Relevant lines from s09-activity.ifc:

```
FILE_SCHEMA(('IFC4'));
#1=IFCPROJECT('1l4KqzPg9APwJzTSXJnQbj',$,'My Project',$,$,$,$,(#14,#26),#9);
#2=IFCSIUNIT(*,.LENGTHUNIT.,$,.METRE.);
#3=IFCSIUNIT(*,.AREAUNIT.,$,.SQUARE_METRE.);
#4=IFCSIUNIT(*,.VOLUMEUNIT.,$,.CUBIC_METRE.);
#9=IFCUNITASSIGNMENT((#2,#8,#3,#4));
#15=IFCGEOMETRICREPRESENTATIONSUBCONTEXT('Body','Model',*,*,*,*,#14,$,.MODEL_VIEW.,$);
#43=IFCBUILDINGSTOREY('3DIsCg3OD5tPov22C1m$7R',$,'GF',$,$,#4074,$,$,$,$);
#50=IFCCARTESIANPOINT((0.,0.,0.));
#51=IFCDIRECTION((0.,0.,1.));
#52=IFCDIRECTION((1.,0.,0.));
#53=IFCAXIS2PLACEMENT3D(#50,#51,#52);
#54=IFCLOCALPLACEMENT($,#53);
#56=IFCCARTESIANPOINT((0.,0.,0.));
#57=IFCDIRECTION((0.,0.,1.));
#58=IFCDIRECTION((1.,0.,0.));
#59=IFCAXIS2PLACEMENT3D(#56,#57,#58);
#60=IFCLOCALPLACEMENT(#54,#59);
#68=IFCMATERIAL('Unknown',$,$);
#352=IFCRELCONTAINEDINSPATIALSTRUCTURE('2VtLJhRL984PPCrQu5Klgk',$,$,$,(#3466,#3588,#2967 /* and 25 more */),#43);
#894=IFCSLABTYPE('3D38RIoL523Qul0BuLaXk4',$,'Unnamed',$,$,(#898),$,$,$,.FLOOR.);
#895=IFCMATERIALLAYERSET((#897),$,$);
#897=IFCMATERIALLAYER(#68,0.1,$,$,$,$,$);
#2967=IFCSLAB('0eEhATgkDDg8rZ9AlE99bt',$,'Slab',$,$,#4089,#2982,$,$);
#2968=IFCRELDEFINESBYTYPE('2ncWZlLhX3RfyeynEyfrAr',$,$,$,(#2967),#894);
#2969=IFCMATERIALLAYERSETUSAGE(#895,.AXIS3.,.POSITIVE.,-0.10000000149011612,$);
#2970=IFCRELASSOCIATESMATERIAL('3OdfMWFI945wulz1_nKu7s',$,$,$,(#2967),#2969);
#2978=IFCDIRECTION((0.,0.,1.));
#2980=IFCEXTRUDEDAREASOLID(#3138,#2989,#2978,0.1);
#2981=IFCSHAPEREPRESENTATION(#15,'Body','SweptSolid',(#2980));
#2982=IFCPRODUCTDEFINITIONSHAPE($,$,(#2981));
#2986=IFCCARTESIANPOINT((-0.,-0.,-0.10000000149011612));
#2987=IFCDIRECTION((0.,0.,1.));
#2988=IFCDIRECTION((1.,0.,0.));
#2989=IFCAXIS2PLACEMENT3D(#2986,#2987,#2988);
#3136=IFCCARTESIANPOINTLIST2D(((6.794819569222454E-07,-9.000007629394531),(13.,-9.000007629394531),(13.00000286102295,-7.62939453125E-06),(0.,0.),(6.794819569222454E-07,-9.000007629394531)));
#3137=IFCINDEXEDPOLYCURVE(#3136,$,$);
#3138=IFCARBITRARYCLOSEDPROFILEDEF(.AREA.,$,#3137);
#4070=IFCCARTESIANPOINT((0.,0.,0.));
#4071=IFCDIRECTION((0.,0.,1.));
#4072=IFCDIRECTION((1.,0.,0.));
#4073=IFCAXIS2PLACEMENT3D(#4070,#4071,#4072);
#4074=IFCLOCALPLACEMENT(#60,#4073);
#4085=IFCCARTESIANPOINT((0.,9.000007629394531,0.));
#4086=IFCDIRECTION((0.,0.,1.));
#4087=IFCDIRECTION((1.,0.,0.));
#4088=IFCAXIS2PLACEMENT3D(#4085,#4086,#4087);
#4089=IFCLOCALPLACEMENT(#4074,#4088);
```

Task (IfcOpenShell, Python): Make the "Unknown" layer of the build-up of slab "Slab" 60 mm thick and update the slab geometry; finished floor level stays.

```python
import ifcopenshell
import ifcopenshell.util.element
import ifcopenshell.util.representation
import ifcopenshell.util.unit

model = ifcopenshell.open("s09-activity.ifc")
unit_scale = ifcopenshell.util.unit.calculate_unit_scale(model)

layer_set = model.by_id(895)
layer = next(l for l in layer_set.MaterialLayers if l.Material and l.Material.Name == "Unknown")
change = 0.06 / unit_scale - layer.LayerThickness
layer.LayerThickness += change

# Geometry does not follow the layer set by itself.
slabs = [e for e in ifcopenshell.util.element.get_elements_by_material(model, layer_set) if e.is_a("IfcSlab")]
for slab in sorted(slabs, key=lambda e: e.id()):
    body = ifcopenshell.util.representation.get_representation(slab, "Model", "Body")
    solid = body.Items[0]
    old_depth = solid.Depth
    solid.Depth += change
    # Extruded upwards: lower the start of the extrusion so the top stays.
    x, y, z = solid.Position.Location.Coordinates
    solid.Position.Location = model.createIfcCartesianPoint((x, y, z - change))
    print(slab.id(), f"{old_depth:g} -> {solid.Depth:g}")

# The layers are counted up from the underside, which has moved.
for usage in {ifcopenshell.util.element.get_material(slab) for slab in slabs}:
    usage.OffsetFromReferenceLine -= change

model.write("s09-activity_rev.ifc")
```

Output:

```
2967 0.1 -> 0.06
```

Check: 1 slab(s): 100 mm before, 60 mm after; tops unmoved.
